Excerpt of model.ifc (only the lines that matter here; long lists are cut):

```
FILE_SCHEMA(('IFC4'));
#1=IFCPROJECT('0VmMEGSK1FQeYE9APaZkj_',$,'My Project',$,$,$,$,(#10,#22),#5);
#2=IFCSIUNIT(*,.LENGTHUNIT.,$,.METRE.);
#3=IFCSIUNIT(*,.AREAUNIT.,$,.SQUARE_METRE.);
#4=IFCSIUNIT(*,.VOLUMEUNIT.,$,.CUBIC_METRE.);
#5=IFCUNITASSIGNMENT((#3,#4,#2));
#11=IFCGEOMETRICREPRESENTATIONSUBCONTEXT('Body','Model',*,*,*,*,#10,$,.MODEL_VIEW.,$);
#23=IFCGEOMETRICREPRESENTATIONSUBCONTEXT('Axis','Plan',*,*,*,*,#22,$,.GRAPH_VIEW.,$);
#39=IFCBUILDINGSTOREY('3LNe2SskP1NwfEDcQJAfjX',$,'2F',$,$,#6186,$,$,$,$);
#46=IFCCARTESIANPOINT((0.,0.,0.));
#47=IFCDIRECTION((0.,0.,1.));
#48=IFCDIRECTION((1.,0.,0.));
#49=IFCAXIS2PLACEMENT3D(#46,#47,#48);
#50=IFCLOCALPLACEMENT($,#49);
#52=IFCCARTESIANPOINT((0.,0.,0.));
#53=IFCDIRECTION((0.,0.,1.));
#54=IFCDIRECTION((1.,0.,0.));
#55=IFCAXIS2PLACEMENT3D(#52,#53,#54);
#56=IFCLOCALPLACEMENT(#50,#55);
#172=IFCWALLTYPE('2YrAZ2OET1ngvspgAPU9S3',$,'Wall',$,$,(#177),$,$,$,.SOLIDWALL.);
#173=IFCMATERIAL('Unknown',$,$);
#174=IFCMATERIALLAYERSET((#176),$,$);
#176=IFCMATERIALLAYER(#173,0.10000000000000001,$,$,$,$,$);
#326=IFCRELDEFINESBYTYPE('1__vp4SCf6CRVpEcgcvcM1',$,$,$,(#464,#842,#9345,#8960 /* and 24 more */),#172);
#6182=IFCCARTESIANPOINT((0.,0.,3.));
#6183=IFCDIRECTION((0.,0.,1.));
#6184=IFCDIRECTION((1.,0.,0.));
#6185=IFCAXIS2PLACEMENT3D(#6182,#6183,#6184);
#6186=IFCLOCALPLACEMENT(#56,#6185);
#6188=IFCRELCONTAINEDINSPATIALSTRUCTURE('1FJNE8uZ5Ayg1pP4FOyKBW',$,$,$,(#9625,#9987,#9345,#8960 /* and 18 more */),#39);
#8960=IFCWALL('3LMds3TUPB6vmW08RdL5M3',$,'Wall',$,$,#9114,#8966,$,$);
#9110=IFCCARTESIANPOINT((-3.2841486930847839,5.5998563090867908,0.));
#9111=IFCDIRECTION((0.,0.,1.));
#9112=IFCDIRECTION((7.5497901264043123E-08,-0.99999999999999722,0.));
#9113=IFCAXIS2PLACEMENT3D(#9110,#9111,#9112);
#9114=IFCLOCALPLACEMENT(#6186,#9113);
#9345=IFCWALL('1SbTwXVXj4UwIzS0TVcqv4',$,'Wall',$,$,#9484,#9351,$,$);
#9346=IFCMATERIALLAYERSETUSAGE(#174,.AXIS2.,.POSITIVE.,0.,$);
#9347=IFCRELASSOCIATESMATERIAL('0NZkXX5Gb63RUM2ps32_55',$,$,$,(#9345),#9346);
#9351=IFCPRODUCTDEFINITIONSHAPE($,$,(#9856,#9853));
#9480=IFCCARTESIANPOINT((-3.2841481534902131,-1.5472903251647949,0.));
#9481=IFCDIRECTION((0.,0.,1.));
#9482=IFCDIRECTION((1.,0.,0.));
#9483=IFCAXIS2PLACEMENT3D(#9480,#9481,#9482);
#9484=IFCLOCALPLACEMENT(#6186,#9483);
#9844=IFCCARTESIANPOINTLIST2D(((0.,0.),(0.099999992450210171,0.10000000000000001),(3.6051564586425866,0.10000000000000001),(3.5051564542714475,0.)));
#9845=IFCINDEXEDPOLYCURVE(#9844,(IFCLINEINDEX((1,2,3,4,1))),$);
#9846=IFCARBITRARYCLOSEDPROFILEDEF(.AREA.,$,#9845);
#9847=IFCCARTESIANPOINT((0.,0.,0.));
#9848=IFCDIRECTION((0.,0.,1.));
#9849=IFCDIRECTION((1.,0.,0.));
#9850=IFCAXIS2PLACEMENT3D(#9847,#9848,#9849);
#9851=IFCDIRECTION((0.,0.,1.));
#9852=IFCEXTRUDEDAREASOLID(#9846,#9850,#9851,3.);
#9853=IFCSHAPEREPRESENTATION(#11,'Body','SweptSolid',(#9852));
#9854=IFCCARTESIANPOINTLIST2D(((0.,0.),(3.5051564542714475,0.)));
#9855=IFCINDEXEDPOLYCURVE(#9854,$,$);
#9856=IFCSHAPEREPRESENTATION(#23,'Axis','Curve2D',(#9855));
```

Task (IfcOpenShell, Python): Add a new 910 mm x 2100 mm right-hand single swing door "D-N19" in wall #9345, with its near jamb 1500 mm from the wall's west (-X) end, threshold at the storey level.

```python
import numpy as np
import ifcopenshell
import ifcopenshell.api.feature
import ifcopenshell.api.geometry
import ifcopenshell.api.root
import ifcopenshell.api.spatial
import ifcopenshell.geom
import ifcopenshell.util.element
import ifcopenshell.util.placement
import ifcopenshell.util.representation
import ifcopenshell.util.shape
import ifcopenshell.util.unit

model = ifcopenshell.open("model.ifc")
unit_scale = ifcopenshell.util.unit.calculate_unit_scale(model)
settings = ifcopenshell.geom.settings()


def volume(element):
    """Net volume in cubic metres, openings subtracted."""
    shape = ifcopenshell.geom.create_shape(settings, element)
    return ifcopenshell.util.shape.get_volume(shape.geometry)


wall = model.by_guid("1SbTwXVXj4UwIzS0TVcqv4")
storey = ifcopenshell.util.element.get_container(wall, ifc_class="IfcBuildingStorey")
context = ifcopenshell.util.representation.get_context(model, "Model", "Body", "MODEL_VIEW")
before = volume(wall)

width, height, from_end, sill = 0.91, 2.1, 1.5, 0.0  # metres

# The wall runs along its own X axis, and the end named is its -X end.
wall_shape = ifcopenshell.geom.create_shape(settings, wall)
x, y, z = ifcopenshell.util.shape.get_vertices(wall_shape.geometry).T
start = x.min() + from_end
face, thickness = float(y.min()), float(y.max() - y.min())
wall_matrix = ifcopenshell.util.placement.get_local_placement(wall.ObjectPlacement)
level = ifcopenshell.util.placement.get_local_placement(storey.ObjectPlacement)[2, 3]


def in_wall(x, y):
    """Placement at x, y metres in the wall's axes, at sill height."""
    matrix = wall_matrix.copy()
    matrix[:, 3] = wall_matrix @ np.array([x / unit_scale, y / unit_scale, 0.0, 1.0])
    matrix[2, 3] = level + sill / unit_scale
    return matrix


# Opening: a box that overshoots both wall faces by 50 mm.
opening = ifcopenshell.api.root.create_entity(model, ifc_class="IfcOpeningElement", predefined_type="OPENING")
box = ifcopenshell.api.geometry.add_wall_representation(
    model, context=context, length=width, height=height, thickness=thickness + 0.1
)
ifcopenshell.api.geometry.assign_representation(model, product=opening, representation=box)
ifcopenshell.api.geometry.edit_object_placement(model, product=opening, matrix=in_wall(start, face - 0.05), is_si=False)
ifcopenshell.api.feature.add_feature(model, feature=opening, element=wall)

door = ifcopenshell.api.root.create_entity(model, ifc_class="IfcDoor", name="D-N19", predefined_type="DOOR")
door.OverallWidth, door.OverallHeight = width / unit_scale, height / unit_scale
door.OperationType = "SINGLE_SWING_RIGHT"
body = ifcopenshell.api.geometry.add_door_representation(
    model,
    context=context,
    overall_width=door.OverallWidth,
    overall_height=door.OverallHeight,
    operation_type="SINGLE_SWING_RIGHT",
    lining_properties={"LiningDepth": thickness / unit_scale, "ThresholdDepth": thickness / unit_scale},
)
ifcopenshell.api.geometry.assign_representation(model, product=door, representation=body)
ifcopenshell.api.spatial.assign_container(model, products=[door], relating_structure=storey)
ifcopenshell.api.feature.add_filling(model, opening=opening, element=door)

# The lining spans the wall, so the door starts at the wall face.
ifcopenshell.api.geometry.edit_object_placement(model, product=door, matrix=in_wall(start, face), is_si=False)

after = volume(wall)

print(f"wall volume {before:.3f} -> {after:.3f} m3")

model.write("model_updated.ifc")
```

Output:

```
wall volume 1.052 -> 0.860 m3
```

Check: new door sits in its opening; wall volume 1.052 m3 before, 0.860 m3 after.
